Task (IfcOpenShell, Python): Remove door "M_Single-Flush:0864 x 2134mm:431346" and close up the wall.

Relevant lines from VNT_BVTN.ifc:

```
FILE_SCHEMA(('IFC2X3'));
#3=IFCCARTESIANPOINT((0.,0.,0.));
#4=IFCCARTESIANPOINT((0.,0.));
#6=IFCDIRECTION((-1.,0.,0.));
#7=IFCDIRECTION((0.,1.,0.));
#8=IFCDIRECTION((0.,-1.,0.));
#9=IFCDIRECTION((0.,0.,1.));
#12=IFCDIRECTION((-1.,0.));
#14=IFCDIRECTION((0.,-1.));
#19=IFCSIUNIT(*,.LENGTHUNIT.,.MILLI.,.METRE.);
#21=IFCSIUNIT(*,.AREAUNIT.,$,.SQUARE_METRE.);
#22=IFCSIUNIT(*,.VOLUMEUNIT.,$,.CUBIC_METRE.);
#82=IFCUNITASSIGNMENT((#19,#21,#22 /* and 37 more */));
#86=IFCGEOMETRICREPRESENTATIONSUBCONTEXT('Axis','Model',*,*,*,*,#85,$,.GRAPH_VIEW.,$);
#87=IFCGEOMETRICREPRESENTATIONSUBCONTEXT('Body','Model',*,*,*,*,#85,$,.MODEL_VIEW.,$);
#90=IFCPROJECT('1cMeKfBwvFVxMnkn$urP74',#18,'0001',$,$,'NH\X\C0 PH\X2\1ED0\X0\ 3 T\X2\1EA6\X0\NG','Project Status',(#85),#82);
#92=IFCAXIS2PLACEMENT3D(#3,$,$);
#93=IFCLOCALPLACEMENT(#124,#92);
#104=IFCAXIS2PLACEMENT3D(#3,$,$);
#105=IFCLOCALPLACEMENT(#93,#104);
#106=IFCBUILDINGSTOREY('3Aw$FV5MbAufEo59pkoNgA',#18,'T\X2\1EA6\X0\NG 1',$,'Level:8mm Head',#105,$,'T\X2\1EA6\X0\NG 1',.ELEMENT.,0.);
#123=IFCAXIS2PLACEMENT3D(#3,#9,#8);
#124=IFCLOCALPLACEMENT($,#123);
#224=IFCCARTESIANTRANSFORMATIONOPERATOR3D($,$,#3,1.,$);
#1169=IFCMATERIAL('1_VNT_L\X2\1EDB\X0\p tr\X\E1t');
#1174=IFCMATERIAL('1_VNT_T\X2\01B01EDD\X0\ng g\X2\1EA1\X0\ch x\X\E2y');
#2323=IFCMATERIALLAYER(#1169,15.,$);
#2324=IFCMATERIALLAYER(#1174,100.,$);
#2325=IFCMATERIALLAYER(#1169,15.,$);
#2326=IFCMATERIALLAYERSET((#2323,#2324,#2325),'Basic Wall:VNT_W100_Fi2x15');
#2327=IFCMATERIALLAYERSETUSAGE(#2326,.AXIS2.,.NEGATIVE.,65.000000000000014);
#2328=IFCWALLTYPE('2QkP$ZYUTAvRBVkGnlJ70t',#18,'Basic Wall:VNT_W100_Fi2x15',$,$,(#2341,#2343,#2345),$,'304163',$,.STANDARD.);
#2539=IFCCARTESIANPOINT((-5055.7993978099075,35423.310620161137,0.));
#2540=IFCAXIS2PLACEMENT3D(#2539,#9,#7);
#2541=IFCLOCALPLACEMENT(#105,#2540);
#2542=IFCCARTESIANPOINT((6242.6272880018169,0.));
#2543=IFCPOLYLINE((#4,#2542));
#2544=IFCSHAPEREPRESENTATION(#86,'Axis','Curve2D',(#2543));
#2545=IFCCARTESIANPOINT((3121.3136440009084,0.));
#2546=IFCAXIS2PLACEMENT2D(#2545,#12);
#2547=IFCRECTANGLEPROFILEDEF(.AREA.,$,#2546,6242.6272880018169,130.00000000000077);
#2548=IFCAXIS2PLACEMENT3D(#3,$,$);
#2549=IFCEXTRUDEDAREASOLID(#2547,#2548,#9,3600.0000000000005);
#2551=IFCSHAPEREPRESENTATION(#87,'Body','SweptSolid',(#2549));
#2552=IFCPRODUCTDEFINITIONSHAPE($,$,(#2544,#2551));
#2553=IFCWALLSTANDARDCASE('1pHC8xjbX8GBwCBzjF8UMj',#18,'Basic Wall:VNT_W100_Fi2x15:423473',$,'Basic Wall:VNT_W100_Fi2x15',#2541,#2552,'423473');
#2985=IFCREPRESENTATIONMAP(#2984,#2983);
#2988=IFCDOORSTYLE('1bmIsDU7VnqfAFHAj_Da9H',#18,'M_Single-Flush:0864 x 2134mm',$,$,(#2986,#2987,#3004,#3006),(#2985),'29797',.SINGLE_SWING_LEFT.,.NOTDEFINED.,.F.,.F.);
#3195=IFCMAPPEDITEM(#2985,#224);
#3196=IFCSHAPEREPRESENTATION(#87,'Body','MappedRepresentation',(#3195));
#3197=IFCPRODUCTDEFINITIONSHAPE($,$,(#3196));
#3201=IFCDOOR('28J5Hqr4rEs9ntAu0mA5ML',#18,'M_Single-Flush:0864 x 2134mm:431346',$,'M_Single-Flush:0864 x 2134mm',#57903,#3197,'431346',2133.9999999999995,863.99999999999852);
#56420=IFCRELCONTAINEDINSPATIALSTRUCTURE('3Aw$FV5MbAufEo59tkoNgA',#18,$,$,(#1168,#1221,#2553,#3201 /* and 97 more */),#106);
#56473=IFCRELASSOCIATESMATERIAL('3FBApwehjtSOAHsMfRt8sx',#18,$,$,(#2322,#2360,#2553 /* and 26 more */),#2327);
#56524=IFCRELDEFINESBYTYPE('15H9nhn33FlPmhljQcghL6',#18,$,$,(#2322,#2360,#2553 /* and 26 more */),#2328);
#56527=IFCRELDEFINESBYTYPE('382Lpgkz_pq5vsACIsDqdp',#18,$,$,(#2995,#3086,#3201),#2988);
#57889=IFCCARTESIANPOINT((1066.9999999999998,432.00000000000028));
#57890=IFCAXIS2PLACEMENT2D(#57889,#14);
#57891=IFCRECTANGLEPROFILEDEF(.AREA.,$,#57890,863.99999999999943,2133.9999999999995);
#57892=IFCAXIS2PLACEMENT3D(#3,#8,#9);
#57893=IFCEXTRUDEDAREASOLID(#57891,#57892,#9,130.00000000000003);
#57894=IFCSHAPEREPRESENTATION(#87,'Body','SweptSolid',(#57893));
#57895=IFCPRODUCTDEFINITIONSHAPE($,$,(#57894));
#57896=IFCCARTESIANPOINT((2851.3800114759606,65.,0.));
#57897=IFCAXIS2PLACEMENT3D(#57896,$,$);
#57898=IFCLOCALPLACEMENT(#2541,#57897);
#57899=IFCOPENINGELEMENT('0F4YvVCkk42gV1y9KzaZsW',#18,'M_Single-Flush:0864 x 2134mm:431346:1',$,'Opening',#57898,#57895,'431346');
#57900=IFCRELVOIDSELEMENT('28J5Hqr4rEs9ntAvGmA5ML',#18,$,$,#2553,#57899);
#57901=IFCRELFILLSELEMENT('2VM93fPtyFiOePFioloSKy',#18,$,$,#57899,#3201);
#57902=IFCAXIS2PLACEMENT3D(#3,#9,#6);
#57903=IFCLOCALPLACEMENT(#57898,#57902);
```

```python
import ifcopenshell
import ifcopenshell.api.feature
import ifcopenshell.api.root
import ifcopenshell.geom
import ifcopenshell.util.shape

model = ifcopenshell.open("VNT_BVTN.ifc")
settings = ifcopenshell.geom.settings()


def volume(element):
    """Net volume in cubic metres, openings subtracted."""
    shape = ifcopenshell.geom.create_shape(settings, element)
    return ifcopenshell.util.shape.get_volume(shape.geometry)


door = model.by_guid("28J5Hqr4rEs9ntAu0mA5ML")
opening = door.FillsVoids[0].RelatingOpeningElement
wall = opening.VoidsElements[0].RelatingBuildingElement
before = volume(wall)

ifcopenshell.api.root.remove_product(model, product=door)
ifcopenshell.api.feature.remove_feature(model, feature=opening)

after = volume(wall)

print(f"wall volume {before:.3f} -> {after:.3f} m3")

model.write("VNT_BVTN_updated.ifc")
```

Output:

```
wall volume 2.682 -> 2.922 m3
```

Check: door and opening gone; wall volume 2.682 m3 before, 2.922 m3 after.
